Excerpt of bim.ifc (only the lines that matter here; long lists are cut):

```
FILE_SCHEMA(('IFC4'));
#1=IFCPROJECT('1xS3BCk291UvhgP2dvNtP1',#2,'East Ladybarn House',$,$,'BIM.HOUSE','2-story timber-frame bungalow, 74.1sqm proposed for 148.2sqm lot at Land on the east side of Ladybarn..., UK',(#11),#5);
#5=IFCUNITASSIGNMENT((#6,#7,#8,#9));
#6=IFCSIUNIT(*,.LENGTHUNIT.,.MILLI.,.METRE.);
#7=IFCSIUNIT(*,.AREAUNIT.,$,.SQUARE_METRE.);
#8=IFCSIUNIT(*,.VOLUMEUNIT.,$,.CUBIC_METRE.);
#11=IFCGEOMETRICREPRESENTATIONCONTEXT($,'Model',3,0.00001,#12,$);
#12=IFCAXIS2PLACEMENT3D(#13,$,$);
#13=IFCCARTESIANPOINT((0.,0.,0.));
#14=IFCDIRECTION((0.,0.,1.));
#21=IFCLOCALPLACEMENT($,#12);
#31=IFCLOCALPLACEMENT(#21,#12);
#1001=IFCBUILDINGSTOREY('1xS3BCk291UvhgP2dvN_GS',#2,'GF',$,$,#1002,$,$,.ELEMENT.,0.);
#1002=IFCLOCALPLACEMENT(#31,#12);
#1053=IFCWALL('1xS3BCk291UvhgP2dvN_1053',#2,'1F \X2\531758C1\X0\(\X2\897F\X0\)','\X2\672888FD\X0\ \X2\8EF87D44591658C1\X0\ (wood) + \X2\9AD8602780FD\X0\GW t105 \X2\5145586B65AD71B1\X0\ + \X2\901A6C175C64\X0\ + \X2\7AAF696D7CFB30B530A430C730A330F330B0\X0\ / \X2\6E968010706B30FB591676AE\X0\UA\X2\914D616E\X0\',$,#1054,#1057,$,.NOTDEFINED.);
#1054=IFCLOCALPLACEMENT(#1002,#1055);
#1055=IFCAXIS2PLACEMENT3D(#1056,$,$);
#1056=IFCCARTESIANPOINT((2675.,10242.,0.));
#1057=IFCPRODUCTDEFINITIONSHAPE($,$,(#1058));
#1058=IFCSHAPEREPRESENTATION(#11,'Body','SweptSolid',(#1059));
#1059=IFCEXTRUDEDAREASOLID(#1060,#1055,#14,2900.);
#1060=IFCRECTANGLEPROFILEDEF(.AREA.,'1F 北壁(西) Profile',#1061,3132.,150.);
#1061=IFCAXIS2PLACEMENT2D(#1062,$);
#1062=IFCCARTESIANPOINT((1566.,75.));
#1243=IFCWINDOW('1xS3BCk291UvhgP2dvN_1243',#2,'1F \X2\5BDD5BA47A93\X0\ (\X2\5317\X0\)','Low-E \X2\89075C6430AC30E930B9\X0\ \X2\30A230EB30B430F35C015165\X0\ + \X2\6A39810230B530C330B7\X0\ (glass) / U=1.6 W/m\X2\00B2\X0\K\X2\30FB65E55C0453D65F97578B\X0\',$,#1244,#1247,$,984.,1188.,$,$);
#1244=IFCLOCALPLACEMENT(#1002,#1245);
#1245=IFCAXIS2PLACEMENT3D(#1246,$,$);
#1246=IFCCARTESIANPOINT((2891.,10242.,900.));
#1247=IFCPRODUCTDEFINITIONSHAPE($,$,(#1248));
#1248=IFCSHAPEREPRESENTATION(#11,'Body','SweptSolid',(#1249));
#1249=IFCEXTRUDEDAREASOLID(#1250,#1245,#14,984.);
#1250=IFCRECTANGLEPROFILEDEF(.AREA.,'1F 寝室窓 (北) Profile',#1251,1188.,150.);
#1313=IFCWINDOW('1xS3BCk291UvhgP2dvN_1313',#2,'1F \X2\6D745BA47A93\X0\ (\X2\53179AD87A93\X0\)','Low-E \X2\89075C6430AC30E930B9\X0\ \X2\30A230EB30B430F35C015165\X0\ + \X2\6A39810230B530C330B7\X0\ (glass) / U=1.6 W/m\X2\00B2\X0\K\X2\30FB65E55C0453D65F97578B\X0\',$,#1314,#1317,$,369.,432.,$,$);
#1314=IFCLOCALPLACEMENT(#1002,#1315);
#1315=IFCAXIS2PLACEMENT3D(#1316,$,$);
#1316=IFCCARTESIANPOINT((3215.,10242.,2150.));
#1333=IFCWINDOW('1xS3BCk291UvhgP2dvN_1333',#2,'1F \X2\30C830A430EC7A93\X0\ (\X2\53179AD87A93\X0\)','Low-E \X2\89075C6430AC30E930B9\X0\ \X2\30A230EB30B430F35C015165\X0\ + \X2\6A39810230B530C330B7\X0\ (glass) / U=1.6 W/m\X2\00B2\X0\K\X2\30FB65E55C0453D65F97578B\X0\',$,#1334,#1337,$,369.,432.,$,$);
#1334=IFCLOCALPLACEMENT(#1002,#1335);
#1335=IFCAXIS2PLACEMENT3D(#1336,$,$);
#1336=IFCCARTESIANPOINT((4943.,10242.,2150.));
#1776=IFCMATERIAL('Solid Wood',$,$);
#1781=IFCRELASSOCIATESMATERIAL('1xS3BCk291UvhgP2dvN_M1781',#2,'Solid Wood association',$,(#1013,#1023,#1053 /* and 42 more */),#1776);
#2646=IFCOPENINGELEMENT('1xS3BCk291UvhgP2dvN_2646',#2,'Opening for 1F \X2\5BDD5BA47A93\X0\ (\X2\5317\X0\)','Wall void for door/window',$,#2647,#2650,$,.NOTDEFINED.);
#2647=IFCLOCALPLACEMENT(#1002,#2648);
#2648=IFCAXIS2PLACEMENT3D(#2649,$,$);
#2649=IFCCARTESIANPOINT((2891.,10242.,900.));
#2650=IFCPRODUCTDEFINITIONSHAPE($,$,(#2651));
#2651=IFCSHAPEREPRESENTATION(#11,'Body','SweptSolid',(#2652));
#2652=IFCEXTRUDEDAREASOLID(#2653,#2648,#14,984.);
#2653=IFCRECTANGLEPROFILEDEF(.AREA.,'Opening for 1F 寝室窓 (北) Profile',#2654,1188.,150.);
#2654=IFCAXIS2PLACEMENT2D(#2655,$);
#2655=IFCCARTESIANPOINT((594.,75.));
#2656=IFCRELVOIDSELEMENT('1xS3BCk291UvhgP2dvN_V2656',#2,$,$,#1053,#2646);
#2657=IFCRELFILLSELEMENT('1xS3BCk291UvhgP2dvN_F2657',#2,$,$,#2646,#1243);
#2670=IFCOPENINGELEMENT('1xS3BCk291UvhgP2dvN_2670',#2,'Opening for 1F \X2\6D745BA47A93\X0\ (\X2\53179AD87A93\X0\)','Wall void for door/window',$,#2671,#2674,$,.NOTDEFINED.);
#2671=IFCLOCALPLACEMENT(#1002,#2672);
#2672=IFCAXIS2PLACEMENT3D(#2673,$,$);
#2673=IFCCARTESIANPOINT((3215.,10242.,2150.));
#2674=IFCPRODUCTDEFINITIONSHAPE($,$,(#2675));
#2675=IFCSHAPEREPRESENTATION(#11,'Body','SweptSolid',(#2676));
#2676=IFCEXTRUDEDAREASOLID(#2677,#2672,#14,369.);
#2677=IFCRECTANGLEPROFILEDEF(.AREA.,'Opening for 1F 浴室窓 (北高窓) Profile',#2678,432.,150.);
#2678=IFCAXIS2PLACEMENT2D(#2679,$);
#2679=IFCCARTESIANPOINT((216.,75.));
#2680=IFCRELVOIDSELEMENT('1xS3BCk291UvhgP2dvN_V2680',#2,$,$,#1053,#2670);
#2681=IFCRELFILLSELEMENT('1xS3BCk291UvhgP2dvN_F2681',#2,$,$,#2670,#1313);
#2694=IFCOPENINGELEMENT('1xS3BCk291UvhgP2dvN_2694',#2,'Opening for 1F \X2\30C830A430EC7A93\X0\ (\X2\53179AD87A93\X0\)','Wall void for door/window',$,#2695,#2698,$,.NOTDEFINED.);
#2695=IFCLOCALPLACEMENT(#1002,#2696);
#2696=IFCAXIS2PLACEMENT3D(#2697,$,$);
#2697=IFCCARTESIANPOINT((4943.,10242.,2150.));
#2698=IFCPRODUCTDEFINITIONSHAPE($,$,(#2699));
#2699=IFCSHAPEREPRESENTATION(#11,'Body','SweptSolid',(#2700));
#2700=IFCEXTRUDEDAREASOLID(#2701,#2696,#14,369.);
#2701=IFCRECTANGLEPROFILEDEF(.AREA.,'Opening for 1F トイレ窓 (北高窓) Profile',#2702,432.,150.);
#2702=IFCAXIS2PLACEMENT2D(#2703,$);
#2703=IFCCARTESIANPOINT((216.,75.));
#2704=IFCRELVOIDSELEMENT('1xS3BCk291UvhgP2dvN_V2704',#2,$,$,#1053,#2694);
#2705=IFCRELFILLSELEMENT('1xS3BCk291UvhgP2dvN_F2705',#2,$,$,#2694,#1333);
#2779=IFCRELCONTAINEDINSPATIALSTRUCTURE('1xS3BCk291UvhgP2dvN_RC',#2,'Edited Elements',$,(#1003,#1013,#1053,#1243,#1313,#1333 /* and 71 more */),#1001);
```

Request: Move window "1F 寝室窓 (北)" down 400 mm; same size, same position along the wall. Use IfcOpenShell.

```python
import numpy as np
import ifcopenshell
import ifcopenshell.api.geometry
import ifcopenshell.util.placement
import ifcopenshell.util.unit

model = ifcopenshell.open("bim.ifc")
unit_scale = ifcopenshell.util.unit.calculate_unit_scale(model)

window = model.by_id(1243)
opening = window.FillsVoids[0].RelatingOpeningElement
dz = -0.4 / unit_scale

shift = np.array([0.0, 0.0, dz])
# The window is not placed relative to its opening, so move both.
for product in (opening, window):
    matrix = ifcopenshell.util.placement.get_local_placement(product.ObjectPlacement)
    matrix[:3, 3] += shift
    ifcopenshell.api.geometry.edit_object_placement(model, product=product, matrix=matrix, is_si=False)

print(f"moved by {dz * unit_scale:+.3f} m")

model.write("bim_rev.ifc")
```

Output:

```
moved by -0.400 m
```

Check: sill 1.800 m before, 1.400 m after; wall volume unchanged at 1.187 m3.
